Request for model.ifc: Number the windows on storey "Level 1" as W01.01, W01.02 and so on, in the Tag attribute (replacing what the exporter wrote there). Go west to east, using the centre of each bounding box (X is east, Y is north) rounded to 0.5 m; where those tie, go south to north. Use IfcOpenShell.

First a look at what the model holds.

```python
import ifcopenshell
import ifcopenshell.util.element
import ifcopenshell.util.placement

model = ifcopenshell.open("model.ifc")
print(model.schema)
storey = next(s for s in model.by_type("IfcBuildingStorey") if s.Name == "Level 1")
windows = [e for e in ifcopenshell.util.element.get_decomposition(storey) if e.is_a("IfcWindow")]
for e in sorted(windows, key=lambda e: e.id()):
    origin = ifcopenshell.util.placement.get_local_placement(e.ObjectPlacement)[:3, 3]
    print(e.id(), e.Tag, e.Name, origin.round(2) + 0.0, sep=" | ")
```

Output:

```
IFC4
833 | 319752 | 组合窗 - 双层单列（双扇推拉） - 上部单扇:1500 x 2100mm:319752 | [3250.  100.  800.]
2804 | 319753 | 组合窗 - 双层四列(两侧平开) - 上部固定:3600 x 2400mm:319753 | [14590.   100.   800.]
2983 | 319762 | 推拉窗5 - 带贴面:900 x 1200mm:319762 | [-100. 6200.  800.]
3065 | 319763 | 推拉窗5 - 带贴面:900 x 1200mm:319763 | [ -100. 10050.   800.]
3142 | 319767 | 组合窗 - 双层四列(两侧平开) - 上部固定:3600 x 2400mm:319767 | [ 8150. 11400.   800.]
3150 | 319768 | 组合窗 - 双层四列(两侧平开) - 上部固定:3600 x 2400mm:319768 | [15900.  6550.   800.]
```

```python
import ifcopenshell
import ifcopenshell.geom
import ifcopenshell.util.element
import ifcopenshell.util.shape

model = ifcopenshell.open("model.ifc")
settings = ifcopenshell.geom.settings()
settings.set("use-world-coords", True)


def centre(element):
    shape = ifcopenshell.geom.create_shape(settings, element)
    return ifcopenshell.util.shape.get_bbox_centroid(shape.geometry)


storey = next(s for s in model.by_type("IfcBuildingStorey") if s.Name == "Level 1")
windows = [e for e in ifcopenshell.util.element.get_decomposition(storey) if e.is_a("IfcWindow")]

# Insertion points can sit at a corner or the storey origin, so sort by the geometry (in metres).
centres = {e: centre(e) for e in windows}
windows.sort(key=lambda e: (round(centres[e][0] / 0.5), centres[e][1]))

for i, e in enumerate(windows, start=1):
    number = f"W01.{i:02d}"
    e.Tag = number
    print(e.id(), number)

model.write("model_edited.ifc")
```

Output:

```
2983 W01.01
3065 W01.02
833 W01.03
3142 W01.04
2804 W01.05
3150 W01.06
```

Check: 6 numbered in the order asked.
